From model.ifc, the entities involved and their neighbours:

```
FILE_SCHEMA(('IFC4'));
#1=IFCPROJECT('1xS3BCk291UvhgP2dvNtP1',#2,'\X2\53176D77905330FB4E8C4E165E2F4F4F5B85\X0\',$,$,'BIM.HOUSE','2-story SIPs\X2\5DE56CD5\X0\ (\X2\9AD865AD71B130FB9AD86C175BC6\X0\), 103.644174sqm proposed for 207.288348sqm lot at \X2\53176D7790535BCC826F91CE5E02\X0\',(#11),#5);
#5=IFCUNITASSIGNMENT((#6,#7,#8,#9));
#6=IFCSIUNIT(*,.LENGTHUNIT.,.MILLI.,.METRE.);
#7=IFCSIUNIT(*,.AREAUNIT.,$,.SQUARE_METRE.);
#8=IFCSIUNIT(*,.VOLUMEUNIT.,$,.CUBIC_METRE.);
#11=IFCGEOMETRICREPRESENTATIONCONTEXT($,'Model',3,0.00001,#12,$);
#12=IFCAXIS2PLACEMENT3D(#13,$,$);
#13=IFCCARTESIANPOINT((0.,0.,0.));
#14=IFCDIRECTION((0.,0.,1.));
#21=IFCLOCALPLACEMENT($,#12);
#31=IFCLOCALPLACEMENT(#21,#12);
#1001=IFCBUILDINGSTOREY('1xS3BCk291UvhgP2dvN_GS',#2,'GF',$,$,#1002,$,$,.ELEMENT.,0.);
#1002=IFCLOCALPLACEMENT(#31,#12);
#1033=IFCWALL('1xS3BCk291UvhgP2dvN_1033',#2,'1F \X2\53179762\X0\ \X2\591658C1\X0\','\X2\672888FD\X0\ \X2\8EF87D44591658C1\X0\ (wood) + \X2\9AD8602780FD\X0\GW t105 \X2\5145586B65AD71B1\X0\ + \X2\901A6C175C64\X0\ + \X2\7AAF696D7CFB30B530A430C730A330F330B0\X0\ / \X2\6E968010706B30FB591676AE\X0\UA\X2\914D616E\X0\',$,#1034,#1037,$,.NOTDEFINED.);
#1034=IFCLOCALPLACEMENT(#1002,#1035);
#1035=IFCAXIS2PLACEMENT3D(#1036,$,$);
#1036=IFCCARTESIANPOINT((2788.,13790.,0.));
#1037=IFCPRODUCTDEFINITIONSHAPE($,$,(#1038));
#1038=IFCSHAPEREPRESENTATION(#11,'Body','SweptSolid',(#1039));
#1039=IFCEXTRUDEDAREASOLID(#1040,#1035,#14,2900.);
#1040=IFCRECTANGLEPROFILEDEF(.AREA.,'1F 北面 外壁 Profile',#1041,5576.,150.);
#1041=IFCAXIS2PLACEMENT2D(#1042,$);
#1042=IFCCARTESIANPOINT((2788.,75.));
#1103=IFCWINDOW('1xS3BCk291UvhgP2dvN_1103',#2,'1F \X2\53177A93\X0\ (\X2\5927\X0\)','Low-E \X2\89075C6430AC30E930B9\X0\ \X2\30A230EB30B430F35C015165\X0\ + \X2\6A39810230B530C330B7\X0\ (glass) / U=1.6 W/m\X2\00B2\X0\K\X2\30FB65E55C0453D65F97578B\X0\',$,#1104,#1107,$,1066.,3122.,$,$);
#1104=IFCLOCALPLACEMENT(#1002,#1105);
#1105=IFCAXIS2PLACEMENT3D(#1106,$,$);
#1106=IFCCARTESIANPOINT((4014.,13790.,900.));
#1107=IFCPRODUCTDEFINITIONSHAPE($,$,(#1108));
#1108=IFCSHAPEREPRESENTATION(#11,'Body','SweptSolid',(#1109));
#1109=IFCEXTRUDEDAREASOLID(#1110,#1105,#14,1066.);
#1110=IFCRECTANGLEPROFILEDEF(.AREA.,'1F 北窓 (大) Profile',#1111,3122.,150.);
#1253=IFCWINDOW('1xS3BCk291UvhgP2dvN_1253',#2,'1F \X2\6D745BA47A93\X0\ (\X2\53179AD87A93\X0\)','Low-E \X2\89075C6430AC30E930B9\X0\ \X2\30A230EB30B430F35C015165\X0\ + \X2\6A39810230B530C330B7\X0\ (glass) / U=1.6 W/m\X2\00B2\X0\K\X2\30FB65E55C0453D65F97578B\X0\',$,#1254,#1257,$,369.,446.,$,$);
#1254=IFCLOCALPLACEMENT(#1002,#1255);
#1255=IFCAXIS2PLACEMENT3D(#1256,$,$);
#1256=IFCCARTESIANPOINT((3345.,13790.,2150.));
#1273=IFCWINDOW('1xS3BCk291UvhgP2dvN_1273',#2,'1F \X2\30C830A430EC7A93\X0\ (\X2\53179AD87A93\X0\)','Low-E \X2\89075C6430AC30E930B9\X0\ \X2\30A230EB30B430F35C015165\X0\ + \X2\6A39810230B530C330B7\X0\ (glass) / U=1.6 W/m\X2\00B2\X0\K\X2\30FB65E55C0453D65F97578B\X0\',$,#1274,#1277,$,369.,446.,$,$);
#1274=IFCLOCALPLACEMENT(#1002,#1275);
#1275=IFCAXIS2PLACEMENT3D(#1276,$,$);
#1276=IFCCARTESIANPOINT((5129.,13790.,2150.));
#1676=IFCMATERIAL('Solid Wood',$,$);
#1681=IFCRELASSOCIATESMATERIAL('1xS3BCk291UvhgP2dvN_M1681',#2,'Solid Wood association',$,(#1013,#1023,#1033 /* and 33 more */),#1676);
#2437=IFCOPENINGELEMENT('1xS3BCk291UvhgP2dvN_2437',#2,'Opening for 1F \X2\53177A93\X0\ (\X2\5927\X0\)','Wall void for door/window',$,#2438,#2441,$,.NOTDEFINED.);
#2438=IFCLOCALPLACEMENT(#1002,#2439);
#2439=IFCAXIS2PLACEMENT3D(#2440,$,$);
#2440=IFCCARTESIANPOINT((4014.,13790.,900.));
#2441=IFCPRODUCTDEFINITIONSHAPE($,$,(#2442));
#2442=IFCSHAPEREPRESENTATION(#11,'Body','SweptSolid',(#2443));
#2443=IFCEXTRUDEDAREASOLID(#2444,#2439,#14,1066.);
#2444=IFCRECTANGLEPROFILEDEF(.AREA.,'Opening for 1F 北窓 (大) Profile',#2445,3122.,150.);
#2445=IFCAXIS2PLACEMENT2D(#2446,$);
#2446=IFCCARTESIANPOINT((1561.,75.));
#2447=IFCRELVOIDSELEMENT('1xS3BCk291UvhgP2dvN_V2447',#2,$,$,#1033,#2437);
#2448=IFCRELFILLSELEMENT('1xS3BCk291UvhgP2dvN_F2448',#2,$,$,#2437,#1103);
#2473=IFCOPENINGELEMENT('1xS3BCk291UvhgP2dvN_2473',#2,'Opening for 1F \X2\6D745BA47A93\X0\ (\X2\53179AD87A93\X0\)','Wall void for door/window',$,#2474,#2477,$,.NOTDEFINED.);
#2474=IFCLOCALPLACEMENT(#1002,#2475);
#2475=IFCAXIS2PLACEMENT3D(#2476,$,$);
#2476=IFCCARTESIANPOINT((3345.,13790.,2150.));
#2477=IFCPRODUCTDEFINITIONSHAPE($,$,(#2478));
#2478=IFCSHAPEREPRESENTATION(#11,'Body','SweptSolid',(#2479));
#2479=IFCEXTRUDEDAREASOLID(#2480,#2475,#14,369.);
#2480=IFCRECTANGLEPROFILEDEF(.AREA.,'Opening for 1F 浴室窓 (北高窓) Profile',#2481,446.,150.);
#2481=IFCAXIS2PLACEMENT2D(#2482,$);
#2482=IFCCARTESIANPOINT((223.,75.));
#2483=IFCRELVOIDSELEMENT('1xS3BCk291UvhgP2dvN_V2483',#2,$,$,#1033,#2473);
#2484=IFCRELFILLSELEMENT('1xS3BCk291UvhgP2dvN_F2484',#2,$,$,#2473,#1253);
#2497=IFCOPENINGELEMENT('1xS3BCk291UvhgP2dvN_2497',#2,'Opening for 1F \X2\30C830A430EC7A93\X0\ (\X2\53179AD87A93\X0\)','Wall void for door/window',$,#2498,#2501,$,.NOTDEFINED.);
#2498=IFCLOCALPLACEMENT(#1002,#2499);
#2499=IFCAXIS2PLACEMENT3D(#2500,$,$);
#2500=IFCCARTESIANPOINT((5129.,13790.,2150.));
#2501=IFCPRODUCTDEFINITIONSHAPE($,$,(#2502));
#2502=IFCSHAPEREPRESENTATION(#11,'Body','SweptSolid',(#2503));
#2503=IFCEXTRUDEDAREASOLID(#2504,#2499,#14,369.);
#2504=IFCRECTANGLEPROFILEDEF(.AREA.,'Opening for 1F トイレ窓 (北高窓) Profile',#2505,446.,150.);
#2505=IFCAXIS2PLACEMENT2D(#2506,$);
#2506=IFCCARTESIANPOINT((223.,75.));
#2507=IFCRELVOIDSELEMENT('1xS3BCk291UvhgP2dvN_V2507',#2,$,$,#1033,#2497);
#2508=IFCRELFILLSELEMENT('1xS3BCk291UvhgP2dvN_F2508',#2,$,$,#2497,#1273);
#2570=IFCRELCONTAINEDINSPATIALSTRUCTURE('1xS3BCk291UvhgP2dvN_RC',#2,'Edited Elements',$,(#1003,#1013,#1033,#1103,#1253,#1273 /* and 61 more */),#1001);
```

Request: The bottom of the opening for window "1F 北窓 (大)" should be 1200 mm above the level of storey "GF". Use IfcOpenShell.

```python
import numpy as np
import ifcopenshell
import ifcopenshell.api.geometry
import ifcopenshell.geom
import ifcopenshell.util.element
import ifcopenshell.util.placement
import ifcopenshell.util.shape
import ifcopenshell.util.unit

model = ifcopenshell.open("model.ifc")
unit_scale = ifcopenshell.util.unit.calculate_unit_scale(model)

window = model.by_guid("1xS3BCk291UvhgP2dvN_1103")
opening = window.FillsVoids[0].RelatingOpeningElement
storey = ifcopenshell.util.element.get_container(window, ifc_class="IfcBuildingStorey")
level = ifcopenshell.util.placement.get_local_placement(storey.ObjectPlacement)[2, 3]

# The opening's origin need not be at the sill, so measure its lowest point.
shape = ifcopenshell.geom.create_shape(ifcopenshell.geom.settings(), opening)
bottom = ifcopenshell.util.shape.get_shape_bottom_elevation(shape, shape.geometry) / unit_scale
dz = level + 1.2 / unit_scale - bottom

shift = np.array([0.0, 0.0, dz])
# The window is not placed relative to its opening, so move both.
for product in (opening, window):
    matrix = ifcopenshell.util.placement.get_local_placement(product.ObjectPlacement)
    matrix[:3, 3] += shift
    ifcopenshell.api.geometry.edit_object_placement(model, product=product, matrix=matrix, is_si=False)

print(f"moved by {dz * unit_scale:+.3f} m")

model.write("model-out.ifc")
```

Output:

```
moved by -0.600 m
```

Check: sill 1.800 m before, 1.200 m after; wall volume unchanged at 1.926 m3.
